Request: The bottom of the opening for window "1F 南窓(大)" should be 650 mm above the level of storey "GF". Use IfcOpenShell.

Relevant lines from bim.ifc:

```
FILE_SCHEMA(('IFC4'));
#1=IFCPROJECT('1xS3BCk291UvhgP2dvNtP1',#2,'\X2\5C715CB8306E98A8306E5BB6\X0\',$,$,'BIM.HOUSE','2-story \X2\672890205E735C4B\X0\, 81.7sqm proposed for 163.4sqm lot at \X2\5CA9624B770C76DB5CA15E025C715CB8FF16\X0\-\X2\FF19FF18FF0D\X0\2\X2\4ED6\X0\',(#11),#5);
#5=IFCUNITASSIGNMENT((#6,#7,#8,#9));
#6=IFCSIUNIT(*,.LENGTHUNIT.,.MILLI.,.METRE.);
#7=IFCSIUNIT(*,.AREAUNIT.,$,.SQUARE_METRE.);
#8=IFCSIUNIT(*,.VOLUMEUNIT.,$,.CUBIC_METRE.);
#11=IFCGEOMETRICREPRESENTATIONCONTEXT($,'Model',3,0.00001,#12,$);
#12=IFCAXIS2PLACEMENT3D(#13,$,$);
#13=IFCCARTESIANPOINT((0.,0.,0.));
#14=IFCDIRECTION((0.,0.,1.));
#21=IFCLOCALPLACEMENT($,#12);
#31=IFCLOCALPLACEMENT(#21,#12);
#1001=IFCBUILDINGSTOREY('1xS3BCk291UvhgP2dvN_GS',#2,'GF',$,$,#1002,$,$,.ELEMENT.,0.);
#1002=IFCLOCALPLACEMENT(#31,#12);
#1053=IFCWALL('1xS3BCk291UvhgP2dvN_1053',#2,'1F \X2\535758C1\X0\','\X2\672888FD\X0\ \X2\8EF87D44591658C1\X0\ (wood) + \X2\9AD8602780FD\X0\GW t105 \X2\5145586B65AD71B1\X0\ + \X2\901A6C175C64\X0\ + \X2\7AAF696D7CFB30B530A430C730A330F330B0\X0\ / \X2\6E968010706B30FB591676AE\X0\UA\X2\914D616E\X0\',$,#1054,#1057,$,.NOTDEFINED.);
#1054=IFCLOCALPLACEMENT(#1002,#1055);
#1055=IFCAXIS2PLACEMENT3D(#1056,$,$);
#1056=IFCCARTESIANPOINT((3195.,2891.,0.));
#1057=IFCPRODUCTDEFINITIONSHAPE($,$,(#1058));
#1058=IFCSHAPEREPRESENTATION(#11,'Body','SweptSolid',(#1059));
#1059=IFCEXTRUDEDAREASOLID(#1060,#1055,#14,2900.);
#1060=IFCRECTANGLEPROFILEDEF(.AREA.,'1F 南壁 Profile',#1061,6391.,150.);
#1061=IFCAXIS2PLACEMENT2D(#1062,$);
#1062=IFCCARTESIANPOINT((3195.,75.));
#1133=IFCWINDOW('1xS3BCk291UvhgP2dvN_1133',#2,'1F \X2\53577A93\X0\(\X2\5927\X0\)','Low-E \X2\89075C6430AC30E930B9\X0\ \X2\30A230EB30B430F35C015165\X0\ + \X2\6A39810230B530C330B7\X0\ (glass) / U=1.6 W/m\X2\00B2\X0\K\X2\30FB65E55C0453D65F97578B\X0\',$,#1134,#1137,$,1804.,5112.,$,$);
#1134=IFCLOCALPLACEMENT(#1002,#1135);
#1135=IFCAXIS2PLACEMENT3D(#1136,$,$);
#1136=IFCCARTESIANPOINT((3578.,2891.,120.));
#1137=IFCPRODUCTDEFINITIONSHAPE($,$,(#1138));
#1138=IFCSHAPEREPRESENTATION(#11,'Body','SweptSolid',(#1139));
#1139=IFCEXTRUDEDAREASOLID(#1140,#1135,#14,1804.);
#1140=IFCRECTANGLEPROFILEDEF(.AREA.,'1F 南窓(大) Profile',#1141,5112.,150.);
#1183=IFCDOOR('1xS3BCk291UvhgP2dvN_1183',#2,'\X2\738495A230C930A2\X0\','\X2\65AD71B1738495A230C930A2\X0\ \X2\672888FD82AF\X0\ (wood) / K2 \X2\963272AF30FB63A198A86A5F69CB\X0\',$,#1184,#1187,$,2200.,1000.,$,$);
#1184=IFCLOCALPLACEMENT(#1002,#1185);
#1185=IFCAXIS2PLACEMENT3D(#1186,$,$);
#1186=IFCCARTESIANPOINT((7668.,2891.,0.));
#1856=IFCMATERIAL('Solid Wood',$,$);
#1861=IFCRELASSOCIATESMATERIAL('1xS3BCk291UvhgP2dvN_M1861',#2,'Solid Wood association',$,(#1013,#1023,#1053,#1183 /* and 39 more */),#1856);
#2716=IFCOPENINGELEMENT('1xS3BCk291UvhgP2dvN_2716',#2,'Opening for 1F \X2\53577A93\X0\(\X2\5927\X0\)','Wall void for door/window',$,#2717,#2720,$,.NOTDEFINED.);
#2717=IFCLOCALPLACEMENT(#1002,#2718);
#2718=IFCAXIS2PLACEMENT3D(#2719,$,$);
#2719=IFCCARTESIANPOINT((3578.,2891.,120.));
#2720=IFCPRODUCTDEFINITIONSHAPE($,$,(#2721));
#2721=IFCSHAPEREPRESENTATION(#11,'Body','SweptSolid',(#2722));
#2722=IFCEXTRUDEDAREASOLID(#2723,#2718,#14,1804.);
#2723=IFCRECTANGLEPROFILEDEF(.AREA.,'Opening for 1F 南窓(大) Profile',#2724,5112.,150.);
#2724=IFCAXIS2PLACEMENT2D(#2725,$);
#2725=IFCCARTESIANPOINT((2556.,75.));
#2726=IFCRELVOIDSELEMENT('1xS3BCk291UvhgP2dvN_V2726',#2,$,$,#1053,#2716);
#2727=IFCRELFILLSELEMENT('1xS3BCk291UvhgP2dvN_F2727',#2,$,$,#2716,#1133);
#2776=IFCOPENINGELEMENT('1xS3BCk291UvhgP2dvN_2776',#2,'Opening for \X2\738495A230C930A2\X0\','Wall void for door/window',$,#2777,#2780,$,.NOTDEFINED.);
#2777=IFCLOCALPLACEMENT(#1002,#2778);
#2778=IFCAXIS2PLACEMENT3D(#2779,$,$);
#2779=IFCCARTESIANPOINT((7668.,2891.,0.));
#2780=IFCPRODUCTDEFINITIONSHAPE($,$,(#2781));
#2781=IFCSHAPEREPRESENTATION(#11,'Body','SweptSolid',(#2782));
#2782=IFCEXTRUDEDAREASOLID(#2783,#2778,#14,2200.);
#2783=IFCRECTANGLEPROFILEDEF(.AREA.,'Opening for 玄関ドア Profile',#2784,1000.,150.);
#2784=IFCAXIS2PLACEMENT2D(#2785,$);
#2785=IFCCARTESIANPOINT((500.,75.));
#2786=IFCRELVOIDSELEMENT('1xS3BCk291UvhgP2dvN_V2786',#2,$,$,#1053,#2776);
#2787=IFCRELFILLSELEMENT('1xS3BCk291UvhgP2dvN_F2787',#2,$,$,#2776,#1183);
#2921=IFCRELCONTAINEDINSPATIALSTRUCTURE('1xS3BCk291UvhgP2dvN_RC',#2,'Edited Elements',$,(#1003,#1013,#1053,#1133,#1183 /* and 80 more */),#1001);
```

```python
import numpy as np
import ifcopenshell
import ifcopenshell.api.geometry
import ifcopenshell.geom
import ifcopenshell.util.element
import ifcopenshell.util.placement
import ifcopenshell.util.shape
import ifcopenshell.util.unit

model = ifcopenshell.open("bim.ifc")
unit_scale = ifcopenshell.util.unit.calculate_unit_scale(model)

window = model.by_id(1133)
opening = window.FillsVoids[0].RelatingOpeningElement
storey = ifcopenshell.util.element.get_container(window, ifc_class="IfcBuildingStorey")
level = ifcopenshell.util.placement.get_local_placement(storey.ObjectPlacement)[2, 3]

# The opening's origin need not be at the sill, so measure its lowest point.
shape = ifcopenshell.geom.create_shape(ifcopenshell.geom.settings(), opening)
bottom = ifcopenshell.util.shape.get_shape_bottom_elevation(shape, shape.geometry) / unit_scale
dz = level + 0.65 / unit_scale - bottom

shift = np.array([0.0, 0.0, dz])
# The window is not placed relative to its opening, so move both.
for product in (opening, window):
    matrix = ifcopenshell.util.placement.get_local_placement(product.ObjectPlacement)
    matrix[:3, 3] += shift
    ifcopenshell.api.geometry.edit_object_placement(model, product=product, matrix=matrix, is_si=False)

print(f"moved by {dz * unit_scale:+.3f} m")

model.write("bim-out.ifc")
```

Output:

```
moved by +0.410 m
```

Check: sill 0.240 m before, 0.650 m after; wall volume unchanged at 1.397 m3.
